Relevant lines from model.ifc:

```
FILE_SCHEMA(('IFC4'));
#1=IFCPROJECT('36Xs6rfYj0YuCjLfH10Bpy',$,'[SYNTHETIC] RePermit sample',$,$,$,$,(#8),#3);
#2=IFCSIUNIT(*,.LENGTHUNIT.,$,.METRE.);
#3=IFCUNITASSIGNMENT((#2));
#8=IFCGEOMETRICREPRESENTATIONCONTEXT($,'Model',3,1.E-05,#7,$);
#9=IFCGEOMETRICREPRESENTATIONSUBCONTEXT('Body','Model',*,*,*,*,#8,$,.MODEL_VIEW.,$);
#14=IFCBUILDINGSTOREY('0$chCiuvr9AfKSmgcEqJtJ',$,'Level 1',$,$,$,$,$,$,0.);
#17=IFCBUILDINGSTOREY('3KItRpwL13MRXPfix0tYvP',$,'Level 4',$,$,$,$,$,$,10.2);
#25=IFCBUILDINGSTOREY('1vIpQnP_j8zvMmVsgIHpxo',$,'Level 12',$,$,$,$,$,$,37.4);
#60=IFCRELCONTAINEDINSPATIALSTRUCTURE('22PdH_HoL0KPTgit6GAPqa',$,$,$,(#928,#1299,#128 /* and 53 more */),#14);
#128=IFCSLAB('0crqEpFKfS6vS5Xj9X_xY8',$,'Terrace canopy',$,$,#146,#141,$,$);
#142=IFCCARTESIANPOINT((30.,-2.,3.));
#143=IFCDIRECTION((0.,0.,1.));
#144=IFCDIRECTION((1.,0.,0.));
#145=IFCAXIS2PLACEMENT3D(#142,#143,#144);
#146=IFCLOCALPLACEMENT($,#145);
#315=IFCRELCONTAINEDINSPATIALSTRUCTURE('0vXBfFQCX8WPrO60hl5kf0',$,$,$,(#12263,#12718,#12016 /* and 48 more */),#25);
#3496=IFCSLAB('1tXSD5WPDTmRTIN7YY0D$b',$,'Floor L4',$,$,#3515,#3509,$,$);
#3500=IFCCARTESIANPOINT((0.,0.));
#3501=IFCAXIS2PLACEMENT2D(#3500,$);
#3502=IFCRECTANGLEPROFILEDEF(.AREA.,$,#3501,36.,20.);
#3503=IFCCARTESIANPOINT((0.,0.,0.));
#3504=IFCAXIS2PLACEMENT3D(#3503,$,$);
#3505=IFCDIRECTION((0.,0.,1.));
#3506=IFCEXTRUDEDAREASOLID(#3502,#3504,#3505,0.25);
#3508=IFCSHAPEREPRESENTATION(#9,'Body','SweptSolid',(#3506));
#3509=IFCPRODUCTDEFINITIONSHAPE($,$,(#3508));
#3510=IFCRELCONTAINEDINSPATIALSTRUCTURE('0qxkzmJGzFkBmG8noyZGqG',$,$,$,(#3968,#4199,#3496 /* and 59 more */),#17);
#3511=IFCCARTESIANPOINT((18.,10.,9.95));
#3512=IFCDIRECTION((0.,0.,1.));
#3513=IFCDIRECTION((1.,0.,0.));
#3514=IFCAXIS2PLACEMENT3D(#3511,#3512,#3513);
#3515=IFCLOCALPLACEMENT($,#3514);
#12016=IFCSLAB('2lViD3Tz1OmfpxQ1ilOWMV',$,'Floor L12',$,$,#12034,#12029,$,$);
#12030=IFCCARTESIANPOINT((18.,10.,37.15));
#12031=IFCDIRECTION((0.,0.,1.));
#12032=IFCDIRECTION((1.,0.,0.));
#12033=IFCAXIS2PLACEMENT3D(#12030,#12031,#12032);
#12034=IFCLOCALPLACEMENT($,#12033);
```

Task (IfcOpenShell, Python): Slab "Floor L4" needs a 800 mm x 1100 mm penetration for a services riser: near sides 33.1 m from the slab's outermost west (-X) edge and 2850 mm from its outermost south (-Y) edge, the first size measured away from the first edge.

```python
import numpy as np
import ifcopenshell
import ifcopenshell.api.feature
import ifcopenshell.api.geometry
import ifcopenshell.api.root
import ifcopenshell.geom
import ifcopenshell.util.placement
import ifcopenshell.util.representation
import ifcopenshell.util.shape
import ifcopenshell.util.unit

model = ifcopenshell.open("model.ifc")
unit_scale = ifcopenshell.util.unit.calculate_unit_scale(model)
settings = ifcopenshell.geom.settings()


def volume(element):
    """Net volume in cubic metres, openings subtracted."""
    shape = ifcopenshell.geom.create_shape(settings, element)
    return ifcopenshell.util.shape.get_volume(shape.geometry)


slab = model.by_guid("1tXSD5WPDTmRTIN7YY0D$b")
before = volume(slab)

# Extent in the slab's own axes, in metres. The edges named are its -X and -Y sides.
slab_shape = ifcopenshell.geom.create_shape(settings, slab)
vertices = ifcopenshell.util.shape.get_vertices(slab_shape.geometry)
x_min, y_min, bottom = vertices.min(axis=0)
top = vertices[:, 2].max()

opening = ifcopenshell.api.root.create_entity(model, ifc_class="IfcOpeningElement", name="Services riser opening", predefined_type="OPENING")
context = ifcopenshell.util.representation.get_context(model, "Model", "Body", "MODEL_VIEW")
width, depth = 0.8, 1.1
outline = [(0.0, 0.0), (width, 0.0), (width, depth), (0.0, depth), (0.0, 0.0)]
# Overshoot both faces by 50 mm so the cut is clean.
shape = ifcopenshell.api.geometry.add_slab_representation(
    model, context=context, depth=top - bottom + 0.1, polyline=outline
)
ifcopenshell.api.geometry.assign_representation(model, product=opening, representation=shape)

matrix = ifcopenshell.util.placement.get_local_placement(slab.ObjectPlacement)
matrix[:, 3] = matrix @ np.append(np.array([x_min + 33.1, y_min + 2.85, bottom - 0.05]) / unit_scale, 1.0)
ifcopenshell.api.geometry.edit_object_placement(model, product=opening, matrix=matrix, is_si=False)
ifcopenshell.api.feature.add_feature(model, feature=opening, element=slab)

after = volume(slab)

print(f"slab volume {before:.3f} -> {after:.3f} m3")

model.write("model_rev.ifc")
```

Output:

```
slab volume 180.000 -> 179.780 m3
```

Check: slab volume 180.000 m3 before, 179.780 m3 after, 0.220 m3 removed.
